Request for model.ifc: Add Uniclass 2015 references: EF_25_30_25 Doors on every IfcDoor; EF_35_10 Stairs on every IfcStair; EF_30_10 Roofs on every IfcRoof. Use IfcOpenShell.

First a look at what the model holds.

```python
import ifcopenshell

model = ifcopenshell.open("model.ifc")
print(model.schema)
print("classifications:", [c.Name for c in model.by_type("IfcClassification")])
for ifc_class in ("IfcDoor", "IfcRoof", "IfcStair", "IfcWall", "IfcWindow"):
    print(ifc_class, len(model.by_type(ifc_class)))
```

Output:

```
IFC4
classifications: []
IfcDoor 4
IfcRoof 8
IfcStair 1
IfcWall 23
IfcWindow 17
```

```python
import ifcopenshell
import ifcopenshell.api.classification

model = ifcopenshell.open("model.ifc")

system = ifcopenshell.api.classification.add_classification(model, classification="Uniclass 2015")

codes = {
    "IfcDoor": ("EF_25_30_25", "Doors"),
    "IfcStair": ("EF_35_10", "Stairs"),
    "IfcRoof": ("EF_30_10", "Roofs"),
}
for ifc_class, (code, name) in codes.items():
    products = model.by_type(ifc_class)
    ifcopenshell.api.classification.add_reference(
        model, products=products, classification=system, identification=code, name=name
    )
    print(code, len(products))

model.write("model-out.ifc")
```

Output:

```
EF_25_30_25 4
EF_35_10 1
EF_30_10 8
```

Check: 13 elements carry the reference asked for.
